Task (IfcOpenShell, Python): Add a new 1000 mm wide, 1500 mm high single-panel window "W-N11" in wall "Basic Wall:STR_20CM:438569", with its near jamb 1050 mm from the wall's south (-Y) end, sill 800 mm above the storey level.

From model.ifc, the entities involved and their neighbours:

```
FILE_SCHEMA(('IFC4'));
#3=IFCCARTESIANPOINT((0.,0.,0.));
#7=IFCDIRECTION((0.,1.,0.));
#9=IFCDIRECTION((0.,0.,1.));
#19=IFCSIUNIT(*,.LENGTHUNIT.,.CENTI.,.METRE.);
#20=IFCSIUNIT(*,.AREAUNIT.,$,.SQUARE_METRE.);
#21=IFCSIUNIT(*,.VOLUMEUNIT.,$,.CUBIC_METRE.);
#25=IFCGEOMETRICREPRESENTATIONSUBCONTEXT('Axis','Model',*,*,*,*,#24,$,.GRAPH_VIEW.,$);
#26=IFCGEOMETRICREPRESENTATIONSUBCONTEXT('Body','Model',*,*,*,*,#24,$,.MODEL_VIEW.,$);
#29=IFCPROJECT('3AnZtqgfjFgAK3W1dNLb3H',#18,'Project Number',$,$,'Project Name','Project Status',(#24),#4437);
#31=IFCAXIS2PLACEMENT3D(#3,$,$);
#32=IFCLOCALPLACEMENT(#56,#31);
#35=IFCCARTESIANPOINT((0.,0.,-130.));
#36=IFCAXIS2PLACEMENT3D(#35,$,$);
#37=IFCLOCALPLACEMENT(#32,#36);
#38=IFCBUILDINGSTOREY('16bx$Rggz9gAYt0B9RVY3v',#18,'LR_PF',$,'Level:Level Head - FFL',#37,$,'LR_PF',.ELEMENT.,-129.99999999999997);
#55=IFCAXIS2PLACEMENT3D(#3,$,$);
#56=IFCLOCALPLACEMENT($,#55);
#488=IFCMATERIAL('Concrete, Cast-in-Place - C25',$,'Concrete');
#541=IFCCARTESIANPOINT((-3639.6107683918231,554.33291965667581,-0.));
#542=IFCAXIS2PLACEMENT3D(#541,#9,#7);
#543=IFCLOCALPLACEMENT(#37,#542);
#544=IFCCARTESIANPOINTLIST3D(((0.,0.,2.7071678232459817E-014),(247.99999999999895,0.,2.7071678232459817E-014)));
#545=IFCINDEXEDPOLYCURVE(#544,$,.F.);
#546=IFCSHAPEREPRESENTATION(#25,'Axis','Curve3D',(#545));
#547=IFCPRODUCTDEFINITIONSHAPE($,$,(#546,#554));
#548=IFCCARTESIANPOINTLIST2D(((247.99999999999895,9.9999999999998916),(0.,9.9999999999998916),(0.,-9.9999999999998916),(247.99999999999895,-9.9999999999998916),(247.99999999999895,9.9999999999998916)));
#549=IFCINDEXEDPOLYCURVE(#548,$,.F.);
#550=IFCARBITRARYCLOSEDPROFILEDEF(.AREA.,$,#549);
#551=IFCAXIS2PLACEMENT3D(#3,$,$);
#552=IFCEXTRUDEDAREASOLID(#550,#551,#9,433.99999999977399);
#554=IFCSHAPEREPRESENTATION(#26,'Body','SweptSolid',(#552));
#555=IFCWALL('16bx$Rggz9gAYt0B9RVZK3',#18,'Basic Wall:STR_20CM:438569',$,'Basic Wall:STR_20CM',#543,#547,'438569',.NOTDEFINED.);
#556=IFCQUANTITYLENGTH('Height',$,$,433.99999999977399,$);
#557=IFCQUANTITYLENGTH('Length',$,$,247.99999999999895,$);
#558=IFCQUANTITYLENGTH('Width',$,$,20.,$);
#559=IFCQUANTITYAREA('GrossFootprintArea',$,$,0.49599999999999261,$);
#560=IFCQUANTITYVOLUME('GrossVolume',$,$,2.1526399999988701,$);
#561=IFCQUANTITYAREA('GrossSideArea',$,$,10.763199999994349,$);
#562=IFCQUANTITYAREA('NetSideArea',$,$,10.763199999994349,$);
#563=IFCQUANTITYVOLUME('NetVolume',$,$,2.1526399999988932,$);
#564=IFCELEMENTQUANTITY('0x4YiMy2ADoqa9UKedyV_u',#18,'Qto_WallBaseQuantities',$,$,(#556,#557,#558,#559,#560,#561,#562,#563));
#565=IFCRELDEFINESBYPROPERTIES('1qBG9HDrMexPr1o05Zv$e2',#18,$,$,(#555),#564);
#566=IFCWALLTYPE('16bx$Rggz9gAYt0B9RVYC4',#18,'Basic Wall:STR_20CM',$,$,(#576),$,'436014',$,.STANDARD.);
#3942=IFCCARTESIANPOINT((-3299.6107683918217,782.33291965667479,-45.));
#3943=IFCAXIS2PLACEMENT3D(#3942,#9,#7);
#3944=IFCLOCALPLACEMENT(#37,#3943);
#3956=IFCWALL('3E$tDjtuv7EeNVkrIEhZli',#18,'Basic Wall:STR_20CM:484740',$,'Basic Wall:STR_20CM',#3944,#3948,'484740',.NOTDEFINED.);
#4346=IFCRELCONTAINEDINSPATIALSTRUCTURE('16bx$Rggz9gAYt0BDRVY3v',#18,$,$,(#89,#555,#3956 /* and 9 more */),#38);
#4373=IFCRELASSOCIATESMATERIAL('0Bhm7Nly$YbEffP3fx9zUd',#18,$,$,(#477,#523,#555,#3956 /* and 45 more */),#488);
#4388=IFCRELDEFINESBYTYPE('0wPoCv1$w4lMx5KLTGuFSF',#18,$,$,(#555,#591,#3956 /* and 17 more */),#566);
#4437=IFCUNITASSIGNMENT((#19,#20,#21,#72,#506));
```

```python
import numpy as np
import ifcopenshell
import ifcopenshell.api.feature
import ifcopenshell.api.geometry
import ifcopenshell.api.pset
import ifcopenshell.api.root
import ifcopenshell.api.spatial
import ifcopenshell.geom
import ifcopenshell.util.element
import ifcopenshell.util.placement
import ifcopenshell.util.representation
import ifcopenshell.util.shape
import ifcopenshell.util.unit

model = ifcopenshell.open("model.ifc")
unit_scale = ifcopenshell.util.unit.calculate_unit_scale(model)
area_scale = ifcopenshell.util.unit.calculate_unit_scale(model, "AREAUNIT")
volume_scale = ifcopenshell.util.unit.calculate_unit_scale(model, "VOLUMEUNIT")
settings = ifcopenshell.geom.settings()


def volume(element):
    """Net volume in cubic metres, openings subtracted."""
    shape = ifcopenshell.geom.create_shape(settings, element)
    return ifcopenshell.util.shape.get_volume(shape.geometry)


wall = model.by_guid("16bx$Rggz9gAYt0B9RVZK3")
storey = ifcopenshell.util.element.get_container(wall, ifc_class="IfcBuildingStorey")
context = ifcopenshell.util.representation.get_context(model, "Model", "Body", "MODEL_VIEW")
before = volume(wall)

width, height, from_end, sill = 1, 1.5, 1.05, 0.8  # metres

# The wall runs along its own X axis, and the end named is its -X end.
wall_shape = ifcopenshell.geom.create_shape(settings, wall)
x, y, z = ifcopenshell.util.shape.get_vertices(wall_shape.geometry).T
start = x.min() + from_end
face, thickness = float(y.min()), float(y.max() - y.min())
wall_matrix = ifcopenshell.util.placement.get_local_placement(wall.ObjectPlacement)
level = ifcopenshell.util.placement.get_local_placement(storey.ObjectPlacement)[2, 3]


def in_wall(x, y):
    """Placement at x, y metres in the wall's axes, at sill height."""
    matrix = wall_matrix.copy()
    matrix[:, 3] = wall_matrix @ np.array([x / unit_scale, y / unit_scale, 0.0, 1.0])
    matrix[2, 3] = level + sill / unit_scale
    return matrix


# Opening: a box that overshoots both wall faces by 50 mm.
opening = ifcopenshell.api.root.create_entity(model, ifc_class="IfcOpeningElement", predefined_type="OPENING")
box = ifcopenshell.api.geometry.add_wall_representation(
    model, context=context, length=width, height=height, thickness=thickness + 0.1
)
ifcopenshell.api.geometry.assign_representation(model, product=opening, representation=box)
ifcopenshell.api.geometry.edit_object_placement(model, product=opening, matrix=in_wall(start, face - 0.05), is_si=False)
ifcopenshell.api.feature.add_feature(model, feature=opening, element=wall)

window = ifcopenshell.api.root.create_entity(model, ifc_class="IfcWindow", name="W-N11", predefined_type="WINDOW")
window.OverallWidth, window.OverallHeight = width / unit_scale, height / unit_scale
window.PartitioningType = "SINGLE_PANEL"
body = ifcopenshell.api.geometry.add_window_representation(
    model,
    context=context,
    overall_width=window.OverallWidth,
    overall_height=window.OverallHeight,
    partition_type="SINGLE_PANEL",
)
ifcopenshell.api.geometry.assign_representation(model, product=window, representation=body)
ifcopenshell.api.spatial.assign_container(model, products=[window], relating_structure=storey)
ifcopenshell.api.feature.add_filling(model, opening=opening, element=window)

# Centre the window in the wall's thickness.
ifcopenshell.api.geometry.edit_object_placement(model, product=window, matrix=in_wall(start, face), is_si=False)
window_shape = ifcopenshell.geom.create_shape(settings, window)
depth = ifcopenshell.util.shape.get_vertices(window_shape.geometry)[:, 1]
offset = face + thickness / 2 - (depth.min() + depth.max()) / 2
ifcopenshell.api.geometry.edit_object_placement(model, product=window, matrix=in_wall(start, offset), is_si=False)

after = volume(wall)

# Update the wall's stored quantities.
qto = model.by_id(ifcopenshell.util.element.get_pset(wall, "Qto_WallBaseQuantities", should_inherit=False)["id"])
ifcopenshell.api.pset.edit_qto(model, qto=qto, properties={
    "NetSideArea": after / thickness / area_scale,
    "NetVolume": after / volume_scale,
})

print(f"wall volume {before:.3f} -> {after:.3f} m3")

model.write("model_v2.ifc")
```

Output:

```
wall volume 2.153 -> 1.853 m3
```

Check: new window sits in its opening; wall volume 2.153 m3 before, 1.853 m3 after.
